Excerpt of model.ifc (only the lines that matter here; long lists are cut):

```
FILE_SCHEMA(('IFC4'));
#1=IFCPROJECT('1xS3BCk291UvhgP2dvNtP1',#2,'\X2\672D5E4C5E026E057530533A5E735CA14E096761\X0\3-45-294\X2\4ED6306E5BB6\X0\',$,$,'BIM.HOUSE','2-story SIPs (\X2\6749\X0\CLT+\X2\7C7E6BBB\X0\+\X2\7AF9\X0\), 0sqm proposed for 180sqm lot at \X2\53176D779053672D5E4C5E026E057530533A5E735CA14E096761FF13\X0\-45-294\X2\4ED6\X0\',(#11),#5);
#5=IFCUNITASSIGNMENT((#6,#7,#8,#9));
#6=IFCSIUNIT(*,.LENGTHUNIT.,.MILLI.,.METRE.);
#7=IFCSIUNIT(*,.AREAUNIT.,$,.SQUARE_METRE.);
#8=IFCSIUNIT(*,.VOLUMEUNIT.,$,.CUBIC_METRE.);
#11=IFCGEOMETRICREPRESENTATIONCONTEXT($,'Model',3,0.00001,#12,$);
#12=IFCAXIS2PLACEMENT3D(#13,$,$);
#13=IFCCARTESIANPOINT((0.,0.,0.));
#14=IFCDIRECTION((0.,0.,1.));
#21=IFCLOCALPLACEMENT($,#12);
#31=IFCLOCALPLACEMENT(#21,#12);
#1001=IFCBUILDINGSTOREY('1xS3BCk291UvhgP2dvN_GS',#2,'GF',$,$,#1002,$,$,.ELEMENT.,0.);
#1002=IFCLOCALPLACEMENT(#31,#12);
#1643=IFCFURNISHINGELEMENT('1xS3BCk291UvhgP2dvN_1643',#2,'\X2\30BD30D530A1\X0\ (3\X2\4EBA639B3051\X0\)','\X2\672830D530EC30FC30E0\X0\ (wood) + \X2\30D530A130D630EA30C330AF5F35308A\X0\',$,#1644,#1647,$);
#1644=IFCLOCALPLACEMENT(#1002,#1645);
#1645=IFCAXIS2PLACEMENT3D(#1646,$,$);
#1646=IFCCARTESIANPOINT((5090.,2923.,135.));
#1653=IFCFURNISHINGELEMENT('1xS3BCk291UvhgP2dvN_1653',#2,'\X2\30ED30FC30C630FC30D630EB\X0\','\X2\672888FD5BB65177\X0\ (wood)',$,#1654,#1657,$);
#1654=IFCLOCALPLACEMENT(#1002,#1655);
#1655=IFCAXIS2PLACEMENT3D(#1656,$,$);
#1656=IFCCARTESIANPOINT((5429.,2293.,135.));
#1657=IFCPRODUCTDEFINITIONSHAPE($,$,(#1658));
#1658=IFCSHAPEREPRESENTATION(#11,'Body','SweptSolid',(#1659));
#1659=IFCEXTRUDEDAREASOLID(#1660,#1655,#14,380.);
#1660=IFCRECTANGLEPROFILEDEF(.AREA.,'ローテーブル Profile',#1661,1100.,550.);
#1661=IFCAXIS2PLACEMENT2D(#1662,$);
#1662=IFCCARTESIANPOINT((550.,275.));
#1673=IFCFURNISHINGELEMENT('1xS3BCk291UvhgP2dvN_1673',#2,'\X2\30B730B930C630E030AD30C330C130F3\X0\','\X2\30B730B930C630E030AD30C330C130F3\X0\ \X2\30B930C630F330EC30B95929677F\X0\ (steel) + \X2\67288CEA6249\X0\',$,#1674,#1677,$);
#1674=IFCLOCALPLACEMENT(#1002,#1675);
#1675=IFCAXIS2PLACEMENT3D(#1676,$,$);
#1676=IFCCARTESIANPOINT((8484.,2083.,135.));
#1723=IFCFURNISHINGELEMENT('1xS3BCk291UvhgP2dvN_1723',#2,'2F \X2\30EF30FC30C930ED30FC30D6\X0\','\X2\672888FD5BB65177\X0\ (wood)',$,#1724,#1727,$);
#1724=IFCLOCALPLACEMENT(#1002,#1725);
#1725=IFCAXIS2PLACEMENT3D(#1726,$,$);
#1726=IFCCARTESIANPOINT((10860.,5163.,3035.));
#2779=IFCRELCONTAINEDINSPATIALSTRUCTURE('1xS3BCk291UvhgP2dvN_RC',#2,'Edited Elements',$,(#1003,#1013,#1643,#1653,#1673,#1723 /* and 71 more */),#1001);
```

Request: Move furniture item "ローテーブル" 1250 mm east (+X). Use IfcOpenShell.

```python
import ifcopenshell
import ifcopenshell.api.geometry
import ifcopenshell.util.placement

model = ifcopenshell.open("model.ifc")

item = model.by_guid("1xS3BCk291UvhgP2dvN_1653")
matrix = ifcopenshell.util.placement.get_local_placement(item.ObjectPlacement)
matrix[0, 3] += 1250.0
ifcopenshell.api.geometry.edit_object_placement(model, product=item, matrix=matrix, is_si=False)

print(ifcopenshell.util.placement.get_local_placement(item.ObjectPlacement).round(3) + 0.0)

model.write("model_rev.ifc")
```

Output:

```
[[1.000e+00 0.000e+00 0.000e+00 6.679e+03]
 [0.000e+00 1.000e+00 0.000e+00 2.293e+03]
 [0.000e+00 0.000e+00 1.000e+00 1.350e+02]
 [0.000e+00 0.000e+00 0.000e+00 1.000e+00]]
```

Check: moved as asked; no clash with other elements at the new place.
